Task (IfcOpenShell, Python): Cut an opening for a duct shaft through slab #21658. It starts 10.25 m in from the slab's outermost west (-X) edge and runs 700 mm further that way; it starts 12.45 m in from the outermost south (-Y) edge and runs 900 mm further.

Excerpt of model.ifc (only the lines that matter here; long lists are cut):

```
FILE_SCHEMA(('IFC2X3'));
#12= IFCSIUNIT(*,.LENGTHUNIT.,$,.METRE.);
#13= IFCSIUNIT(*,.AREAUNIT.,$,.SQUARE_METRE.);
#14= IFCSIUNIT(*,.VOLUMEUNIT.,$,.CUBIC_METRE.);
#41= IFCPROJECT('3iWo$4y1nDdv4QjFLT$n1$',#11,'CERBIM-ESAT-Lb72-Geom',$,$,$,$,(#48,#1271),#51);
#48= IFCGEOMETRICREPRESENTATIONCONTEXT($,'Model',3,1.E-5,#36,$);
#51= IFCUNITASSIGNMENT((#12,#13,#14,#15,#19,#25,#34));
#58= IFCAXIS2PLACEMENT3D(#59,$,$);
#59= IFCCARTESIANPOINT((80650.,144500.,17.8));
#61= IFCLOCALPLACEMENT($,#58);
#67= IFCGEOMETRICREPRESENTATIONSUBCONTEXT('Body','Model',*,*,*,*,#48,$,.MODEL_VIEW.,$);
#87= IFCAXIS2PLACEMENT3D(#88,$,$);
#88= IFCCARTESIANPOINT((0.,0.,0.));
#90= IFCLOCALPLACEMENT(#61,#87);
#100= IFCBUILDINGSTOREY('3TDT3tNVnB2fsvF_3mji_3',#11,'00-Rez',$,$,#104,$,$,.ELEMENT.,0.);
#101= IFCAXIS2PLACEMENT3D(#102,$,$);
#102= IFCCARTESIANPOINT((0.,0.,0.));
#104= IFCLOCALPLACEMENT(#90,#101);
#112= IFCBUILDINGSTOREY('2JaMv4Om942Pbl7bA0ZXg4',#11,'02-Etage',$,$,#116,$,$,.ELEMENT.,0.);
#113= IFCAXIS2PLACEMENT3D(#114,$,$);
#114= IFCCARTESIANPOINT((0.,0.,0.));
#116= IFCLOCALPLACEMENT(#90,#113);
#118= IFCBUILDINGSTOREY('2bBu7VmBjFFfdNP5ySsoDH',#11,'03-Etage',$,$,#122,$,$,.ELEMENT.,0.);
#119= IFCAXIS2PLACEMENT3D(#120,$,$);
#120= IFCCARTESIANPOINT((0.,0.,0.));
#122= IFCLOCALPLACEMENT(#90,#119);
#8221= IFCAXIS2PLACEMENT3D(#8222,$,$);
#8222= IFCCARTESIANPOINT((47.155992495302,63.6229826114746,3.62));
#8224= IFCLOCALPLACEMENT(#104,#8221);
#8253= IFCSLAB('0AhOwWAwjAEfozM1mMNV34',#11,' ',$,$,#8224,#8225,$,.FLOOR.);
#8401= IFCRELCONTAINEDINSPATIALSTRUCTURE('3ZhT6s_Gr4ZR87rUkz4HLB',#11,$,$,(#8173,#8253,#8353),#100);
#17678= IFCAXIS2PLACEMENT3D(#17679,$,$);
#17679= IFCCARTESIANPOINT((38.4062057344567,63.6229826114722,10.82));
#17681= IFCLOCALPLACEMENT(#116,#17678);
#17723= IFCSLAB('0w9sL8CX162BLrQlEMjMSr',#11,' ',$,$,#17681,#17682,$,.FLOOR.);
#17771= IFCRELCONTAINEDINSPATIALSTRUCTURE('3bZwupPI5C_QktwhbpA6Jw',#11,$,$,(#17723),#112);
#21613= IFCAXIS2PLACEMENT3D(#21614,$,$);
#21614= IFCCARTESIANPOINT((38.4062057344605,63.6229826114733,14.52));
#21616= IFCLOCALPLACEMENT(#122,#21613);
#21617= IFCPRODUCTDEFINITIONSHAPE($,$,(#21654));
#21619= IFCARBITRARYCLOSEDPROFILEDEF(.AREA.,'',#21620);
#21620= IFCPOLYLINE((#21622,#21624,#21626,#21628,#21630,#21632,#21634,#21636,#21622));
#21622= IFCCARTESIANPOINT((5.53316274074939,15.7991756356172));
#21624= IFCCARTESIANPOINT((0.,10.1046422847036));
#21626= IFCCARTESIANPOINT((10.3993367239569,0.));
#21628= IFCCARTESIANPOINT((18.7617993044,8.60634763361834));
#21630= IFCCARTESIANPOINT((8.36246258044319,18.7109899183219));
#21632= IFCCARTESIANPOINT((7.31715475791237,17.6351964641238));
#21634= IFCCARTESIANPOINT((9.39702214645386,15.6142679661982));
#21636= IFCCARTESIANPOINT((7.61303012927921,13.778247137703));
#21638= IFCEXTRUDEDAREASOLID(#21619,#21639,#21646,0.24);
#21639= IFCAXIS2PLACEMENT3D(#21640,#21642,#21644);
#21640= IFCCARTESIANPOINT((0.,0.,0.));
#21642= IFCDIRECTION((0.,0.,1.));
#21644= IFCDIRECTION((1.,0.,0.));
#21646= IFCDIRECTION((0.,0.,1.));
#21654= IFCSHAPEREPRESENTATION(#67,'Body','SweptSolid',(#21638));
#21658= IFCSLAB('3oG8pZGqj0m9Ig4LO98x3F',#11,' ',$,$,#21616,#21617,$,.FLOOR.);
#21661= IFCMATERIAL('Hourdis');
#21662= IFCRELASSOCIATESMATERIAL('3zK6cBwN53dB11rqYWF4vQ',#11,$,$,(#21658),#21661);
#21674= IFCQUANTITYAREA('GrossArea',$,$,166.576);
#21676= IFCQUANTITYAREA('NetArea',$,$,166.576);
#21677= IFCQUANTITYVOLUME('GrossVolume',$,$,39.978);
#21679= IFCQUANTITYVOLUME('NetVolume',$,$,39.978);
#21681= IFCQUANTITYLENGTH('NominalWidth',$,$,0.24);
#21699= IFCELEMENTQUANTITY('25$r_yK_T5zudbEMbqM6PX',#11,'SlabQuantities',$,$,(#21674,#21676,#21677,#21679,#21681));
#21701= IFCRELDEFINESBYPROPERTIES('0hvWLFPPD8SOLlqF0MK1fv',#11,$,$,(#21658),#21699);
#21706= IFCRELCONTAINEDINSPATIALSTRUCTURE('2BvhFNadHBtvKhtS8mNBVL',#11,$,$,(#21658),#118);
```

```python
import numpy as np
import ifcopenshell
import ifcopenshell.api.feature
import ifcopenshell.api.geometry
import ifcopenshell.api.pset
import ifcopenshell.api.root
import ifcopenshell.geom
import ifcopenshell.util.element
import ifcopenshell.util.placement
import ifcopenshell.util.representation
import ifcopenshell.util.shape
import ifcopenshell.util.unit

model = ifcopenshell.open("model.ifc")
unit_scale = ifcopenshell.util.unit.calculate_unit_scale(model)
area_scale = ifcopenshell.util.unit.calculate_unit_scale(model, "AREAUNIT")
volume_scale = ifcopenshell.util.unit.calculate_unit_scale(model, "VOLUMEUNIT")
settings = ifcopenshell.geom.settings()


def volume(element):
    """Net volume in cubic metres, openings subtracted."""
    shape = ifcopenshell.geom.create_shape(settings, element)
    return ifcopenshell.util.shape.get_volume(shape.geometry)


slab = model.by_id(21658)
before = volume(slab)

# Extent in the slab's own axes, in metres. The edges named are its -X and -Y sides.
slab_shape = ifcopenshell.geom.create_shape(settings, slab)
vertices = ifcopenshell.util.shape.get_vertices(slab_shape.geometry)
x_min, y_min, bottom = vertices.min(axis=0)
top = vertices[:, 2].max()

opening = ifcopenshell.api.root.create_entity(model, ifc_class="IfcOpeningElement", name="Duct shaft opening")
context = ifcopenshell.util.representation.get_context(model, "Model", "Body", "MODEL_VIEW")
width, depth = 0.7, 0.9
outline = [(0.0, 0.0), (width, 0.0), (width, depth), (0.0, depth), (0.0, 0.0)]
# Overshoot both faces by 50 mm so the cut is clean.
shape = ifcopenshell.api.geometry.add_slab_representation(
    model, context=context, depth=top - bottom + 0.1, polyline=outline
)
ifcopenshell.api.geometry.assign_representation(model, product=opening, representation=shape)

matrix = ifcopenshell.util.placement.get_local_placement(slab.ObjectPlacement)
matrix[:, 3] = matrix @ np.append(np.array([x_min + 10.25, y_min + 12.45, bottom - 0.05]) / unit_scale, 1.0)
ifcopenshell.api.geometry.edit_object_placement(model, product=opening, matrix=matrix, is_si=False)
ifcopenshell.api.feature.add_feature(model, feature=opening, element=slab)

after = volume(slab)

# Update the slab's stored quantities.
qto = model.by_id(ifcopenshell.util.element.get_pset(slab, "SlabQuantities", should_inherit=False)["id"])
ifcopenshell.api.pset.edit_qto(model, qto=qto, properties={
    "NetArea": after / (top - bottom) / area_scale,
    "NetVolume": after / volume_scale,
})

print(f"slab volume {before:.3f} -> {after:.3f} m3")

model.write("model_edited.ifc")
```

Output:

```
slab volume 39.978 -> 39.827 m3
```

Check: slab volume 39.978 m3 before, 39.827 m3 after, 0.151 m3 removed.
